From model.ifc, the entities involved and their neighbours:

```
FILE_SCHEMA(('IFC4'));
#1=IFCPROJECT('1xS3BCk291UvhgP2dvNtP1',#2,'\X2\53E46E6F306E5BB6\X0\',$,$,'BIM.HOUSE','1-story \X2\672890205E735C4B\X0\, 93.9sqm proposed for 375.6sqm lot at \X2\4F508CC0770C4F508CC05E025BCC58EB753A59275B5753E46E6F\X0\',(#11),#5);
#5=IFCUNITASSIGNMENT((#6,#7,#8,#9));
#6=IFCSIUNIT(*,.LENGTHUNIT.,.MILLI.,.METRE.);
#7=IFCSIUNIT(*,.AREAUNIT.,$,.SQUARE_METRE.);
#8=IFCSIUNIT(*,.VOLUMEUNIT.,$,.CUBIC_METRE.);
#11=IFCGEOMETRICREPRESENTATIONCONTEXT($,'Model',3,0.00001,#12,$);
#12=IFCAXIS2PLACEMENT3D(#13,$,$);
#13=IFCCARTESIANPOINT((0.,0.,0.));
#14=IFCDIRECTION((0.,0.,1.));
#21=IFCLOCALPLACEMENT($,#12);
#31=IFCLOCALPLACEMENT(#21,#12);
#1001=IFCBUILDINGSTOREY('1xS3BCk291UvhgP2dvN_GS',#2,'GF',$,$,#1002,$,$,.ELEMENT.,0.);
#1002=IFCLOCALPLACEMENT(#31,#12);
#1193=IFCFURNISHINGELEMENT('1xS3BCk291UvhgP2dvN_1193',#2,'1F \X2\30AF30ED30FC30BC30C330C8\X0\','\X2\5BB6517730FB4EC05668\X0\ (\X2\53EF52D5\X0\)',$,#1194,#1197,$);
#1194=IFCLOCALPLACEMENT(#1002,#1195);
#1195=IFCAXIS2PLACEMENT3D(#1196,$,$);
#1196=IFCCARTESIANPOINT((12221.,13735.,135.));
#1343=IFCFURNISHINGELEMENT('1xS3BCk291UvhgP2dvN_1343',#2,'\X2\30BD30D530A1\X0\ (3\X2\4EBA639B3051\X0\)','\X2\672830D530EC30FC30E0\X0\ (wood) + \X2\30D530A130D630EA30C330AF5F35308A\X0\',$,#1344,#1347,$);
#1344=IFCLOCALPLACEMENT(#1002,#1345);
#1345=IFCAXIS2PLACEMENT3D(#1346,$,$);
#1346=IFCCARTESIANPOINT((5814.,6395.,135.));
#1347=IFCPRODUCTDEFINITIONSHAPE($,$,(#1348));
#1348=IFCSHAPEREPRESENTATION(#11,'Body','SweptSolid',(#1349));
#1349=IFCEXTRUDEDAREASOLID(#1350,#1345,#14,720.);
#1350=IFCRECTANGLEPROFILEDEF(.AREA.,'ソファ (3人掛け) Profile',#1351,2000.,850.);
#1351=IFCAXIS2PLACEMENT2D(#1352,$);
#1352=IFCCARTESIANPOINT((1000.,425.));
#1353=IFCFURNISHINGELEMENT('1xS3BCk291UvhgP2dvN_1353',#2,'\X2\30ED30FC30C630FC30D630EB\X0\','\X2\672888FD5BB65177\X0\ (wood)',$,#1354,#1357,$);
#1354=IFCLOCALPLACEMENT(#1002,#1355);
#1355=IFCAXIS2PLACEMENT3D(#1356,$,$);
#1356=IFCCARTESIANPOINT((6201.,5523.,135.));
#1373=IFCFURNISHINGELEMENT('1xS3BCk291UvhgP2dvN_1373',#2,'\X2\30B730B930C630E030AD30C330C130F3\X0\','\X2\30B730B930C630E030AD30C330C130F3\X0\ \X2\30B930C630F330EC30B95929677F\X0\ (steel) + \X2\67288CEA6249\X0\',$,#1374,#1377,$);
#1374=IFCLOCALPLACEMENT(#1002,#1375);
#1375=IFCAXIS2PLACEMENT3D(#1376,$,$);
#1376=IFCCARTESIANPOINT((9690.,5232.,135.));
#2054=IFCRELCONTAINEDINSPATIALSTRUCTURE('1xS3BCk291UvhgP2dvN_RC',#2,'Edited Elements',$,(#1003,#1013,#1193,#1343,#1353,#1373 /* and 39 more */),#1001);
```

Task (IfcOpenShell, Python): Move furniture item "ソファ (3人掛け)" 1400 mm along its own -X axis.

```python
import ifcopenshell
import ifcopenshell.api.geometry
import ifcopenshell.util.placement
import ifcopenshell.util.unit

model = ifcopenshell.open("model.ifc")
unit_scale = ifcopenshell.util.unit.calculate_unit_scale(model)

item = model.by_id(1343)
matrix = ifcopenshell.util.placement.get_local_placement(item.ObjectPlacement)
matrix[:3, 3] -= matrix[:3, 0] * 1.4 / unit_scale
ifcopenshell.api.geometry.edit_object_placement(model, product=item, matrix=matrix, is_si=False)

print(ifcopenshell.util.placement.get_local_placement(item.ObjectPlacement).round(3) + 0.0)

model.write("model-out.ifc")
```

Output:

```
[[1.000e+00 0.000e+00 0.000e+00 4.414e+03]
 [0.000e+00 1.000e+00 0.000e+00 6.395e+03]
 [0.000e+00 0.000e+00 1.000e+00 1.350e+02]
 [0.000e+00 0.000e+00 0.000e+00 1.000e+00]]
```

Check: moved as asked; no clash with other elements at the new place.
